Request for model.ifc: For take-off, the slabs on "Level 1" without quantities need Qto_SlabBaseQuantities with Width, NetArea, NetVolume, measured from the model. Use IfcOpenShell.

First a look at what the model holds.

```python
import ifcopenshell
import ifcopenshell.util.element
import ifcopenshell.util.unit

model = ifcopenshell.open("model.ifc")
print(model.schema)
for unit_type in ("LENGTHUNIT", "AREAUNIT", "VOLUMEUNIT"):
    print(unit_type, ifcopenshell.util.unit.calculate_unit_scale(model, unit_type))
storey = next(s for s in model.by_type("IfcBuildingStorey") if s.Name == "Level 1")
slabs = [e for e in ifcopenshell.util.element.get_decomposition(storey) if e.is_a("IfcSlab")]
for e in sorted(slabs, key=lambda e: e.id()):
    print(e.id(), e.is_a(), e.Name, list(ifcopenshell.util.element.get_psets(e, qtos_only=True)), sep=" | ")
```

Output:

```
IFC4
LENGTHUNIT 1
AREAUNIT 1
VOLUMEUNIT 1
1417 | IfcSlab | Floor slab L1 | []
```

```python
import ifcopenshell
import ifcopenshell.api.pset
import ifcopenshell.geom
import ifcopenshell.util.element
import ifcopenshell.util.shape
import ifcopenshell.util.unit

model = ifcopenshell.open("model.ifc")
unit_scale = ifcopenshell.util.unit.calculate_unit_scale(model)
area_scale = ifcopenshell.util.unit.calculate_unit_scale(model, "AREAUNIT")
volume_scale = ifcopenshell.util.unit.calculate_unit_scale(model, "VOLUMEUNIT")
settings = ifcopenshell.geom.settings()

storey = next(s for s in model.by_type("IfcBuildingStorey") if s.Name == "Level 1")
slabs = [e for e in ifcopenshell.util.element.get_decomposition(storey) if e.is_a("IfcSlab")]

for e in sorted(slabs, key=lambda e: e.id()):
    if ifcopenshell.util.element.get_psets(e, qtos_only=True, should_inherit=False):
        continue
    # Geometry comes back in metres, in the element's own axes.
    shape = ifcopenshell.geom.create_shape(settings, e)
    values = {
        "Width": ifcopenshell.util.shape.get_z(shape.geometry) / unit_scale,
        "NetArea": ifcopenshell.util.shape.get_footprint_area(shape.geometry) / area_scale,
        "NetVolume": ifcopenshell.util.shape.get_volume(shape.geometry) / volume_scale,
    }
    qto = ifcopenshell.api.pset.add_qto(model, product=e, name="Qto_SlabBaseQuantities")
    ifcopenshell.api.pset.edit_qto(model, qto=qto, properties=values)
    print(e.id(), {k: round(v, 3) for k, v in values.items()})

model.write("model_updated.ifc")
```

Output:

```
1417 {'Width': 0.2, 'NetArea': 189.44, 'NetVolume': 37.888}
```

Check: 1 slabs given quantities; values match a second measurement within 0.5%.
